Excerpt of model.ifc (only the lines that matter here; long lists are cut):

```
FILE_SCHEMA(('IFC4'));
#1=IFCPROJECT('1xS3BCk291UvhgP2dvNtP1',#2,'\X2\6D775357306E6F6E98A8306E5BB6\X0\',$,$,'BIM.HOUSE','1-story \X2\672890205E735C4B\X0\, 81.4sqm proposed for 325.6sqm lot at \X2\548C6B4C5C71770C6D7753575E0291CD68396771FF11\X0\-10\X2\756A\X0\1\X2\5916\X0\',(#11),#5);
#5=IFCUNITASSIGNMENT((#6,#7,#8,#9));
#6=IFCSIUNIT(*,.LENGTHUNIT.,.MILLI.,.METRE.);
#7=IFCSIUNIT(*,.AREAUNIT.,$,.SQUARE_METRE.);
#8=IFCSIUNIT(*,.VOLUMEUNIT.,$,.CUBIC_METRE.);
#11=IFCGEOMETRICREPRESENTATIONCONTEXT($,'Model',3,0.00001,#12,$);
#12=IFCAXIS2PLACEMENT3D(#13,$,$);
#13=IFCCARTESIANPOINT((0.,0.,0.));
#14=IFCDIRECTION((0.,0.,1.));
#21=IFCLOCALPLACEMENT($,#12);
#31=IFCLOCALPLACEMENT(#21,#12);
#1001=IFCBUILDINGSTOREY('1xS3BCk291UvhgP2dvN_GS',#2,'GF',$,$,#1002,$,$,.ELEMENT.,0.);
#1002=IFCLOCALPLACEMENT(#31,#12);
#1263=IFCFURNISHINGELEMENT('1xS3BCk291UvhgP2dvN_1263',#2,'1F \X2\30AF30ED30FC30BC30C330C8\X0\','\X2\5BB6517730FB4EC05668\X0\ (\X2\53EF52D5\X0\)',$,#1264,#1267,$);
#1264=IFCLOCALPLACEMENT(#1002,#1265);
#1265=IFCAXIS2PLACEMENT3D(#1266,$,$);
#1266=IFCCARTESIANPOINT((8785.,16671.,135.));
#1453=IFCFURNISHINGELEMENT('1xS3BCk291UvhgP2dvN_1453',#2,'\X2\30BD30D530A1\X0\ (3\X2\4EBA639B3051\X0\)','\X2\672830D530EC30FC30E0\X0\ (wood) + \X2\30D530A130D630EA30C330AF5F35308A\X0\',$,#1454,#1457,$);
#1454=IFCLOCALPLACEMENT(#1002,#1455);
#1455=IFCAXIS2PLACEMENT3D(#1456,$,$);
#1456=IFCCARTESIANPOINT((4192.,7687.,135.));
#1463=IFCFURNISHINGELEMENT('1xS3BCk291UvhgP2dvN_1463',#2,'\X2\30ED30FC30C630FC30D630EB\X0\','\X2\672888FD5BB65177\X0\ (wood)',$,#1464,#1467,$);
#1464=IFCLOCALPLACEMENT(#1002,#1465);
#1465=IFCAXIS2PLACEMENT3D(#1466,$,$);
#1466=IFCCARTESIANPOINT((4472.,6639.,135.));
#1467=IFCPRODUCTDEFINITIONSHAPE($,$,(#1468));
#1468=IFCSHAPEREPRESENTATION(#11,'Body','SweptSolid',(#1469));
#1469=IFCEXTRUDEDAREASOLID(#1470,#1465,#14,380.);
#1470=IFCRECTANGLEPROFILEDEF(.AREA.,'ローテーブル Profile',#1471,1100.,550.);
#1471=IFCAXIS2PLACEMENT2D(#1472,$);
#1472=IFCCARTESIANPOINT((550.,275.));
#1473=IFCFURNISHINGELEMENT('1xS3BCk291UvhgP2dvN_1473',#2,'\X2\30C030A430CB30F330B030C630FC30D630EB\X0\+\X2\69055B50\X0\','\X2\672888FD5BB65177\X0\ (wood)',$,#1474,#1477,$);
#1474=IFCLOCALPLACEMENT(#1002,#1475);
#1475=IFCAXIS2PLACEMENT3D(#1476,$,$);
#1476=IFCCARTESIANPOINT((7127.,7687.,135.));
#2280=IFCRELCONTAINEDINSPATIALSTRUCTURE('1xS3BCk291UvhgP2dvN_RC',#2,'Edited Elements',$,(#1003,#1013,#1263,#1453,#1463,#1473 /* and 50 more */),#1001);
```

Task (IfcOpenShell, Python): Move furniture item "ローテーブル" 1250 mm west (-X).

```python
import ifcopenshell
import ifcopenshell.api.geometry
import ifcopenshell.util.placement

model = ifcopenshell.open("model.ifc")

item = model.by_id(1463)
matrix = ifcopenshell.util.placement.get_local_placement(item.ObjectPlacement)
matrix[0, 3] -= 1250.0
ifcopenshell.api.geometry.edit_object_placement(model, product=item, matrix=matrix, is_si=False)

print(ifcopenshell.util.placement.get_local_placement(item.ObjectPlacement).round(3) + 0.0)

model.write("model_v2.ifc")
```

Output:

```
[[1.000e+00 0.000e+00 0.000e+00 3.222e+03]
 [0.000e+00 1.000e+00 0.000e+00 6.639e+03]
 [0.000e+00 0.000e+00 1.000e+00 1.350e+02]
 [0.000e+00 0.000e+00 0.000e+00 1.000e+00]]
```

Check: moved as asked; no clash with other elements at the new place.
